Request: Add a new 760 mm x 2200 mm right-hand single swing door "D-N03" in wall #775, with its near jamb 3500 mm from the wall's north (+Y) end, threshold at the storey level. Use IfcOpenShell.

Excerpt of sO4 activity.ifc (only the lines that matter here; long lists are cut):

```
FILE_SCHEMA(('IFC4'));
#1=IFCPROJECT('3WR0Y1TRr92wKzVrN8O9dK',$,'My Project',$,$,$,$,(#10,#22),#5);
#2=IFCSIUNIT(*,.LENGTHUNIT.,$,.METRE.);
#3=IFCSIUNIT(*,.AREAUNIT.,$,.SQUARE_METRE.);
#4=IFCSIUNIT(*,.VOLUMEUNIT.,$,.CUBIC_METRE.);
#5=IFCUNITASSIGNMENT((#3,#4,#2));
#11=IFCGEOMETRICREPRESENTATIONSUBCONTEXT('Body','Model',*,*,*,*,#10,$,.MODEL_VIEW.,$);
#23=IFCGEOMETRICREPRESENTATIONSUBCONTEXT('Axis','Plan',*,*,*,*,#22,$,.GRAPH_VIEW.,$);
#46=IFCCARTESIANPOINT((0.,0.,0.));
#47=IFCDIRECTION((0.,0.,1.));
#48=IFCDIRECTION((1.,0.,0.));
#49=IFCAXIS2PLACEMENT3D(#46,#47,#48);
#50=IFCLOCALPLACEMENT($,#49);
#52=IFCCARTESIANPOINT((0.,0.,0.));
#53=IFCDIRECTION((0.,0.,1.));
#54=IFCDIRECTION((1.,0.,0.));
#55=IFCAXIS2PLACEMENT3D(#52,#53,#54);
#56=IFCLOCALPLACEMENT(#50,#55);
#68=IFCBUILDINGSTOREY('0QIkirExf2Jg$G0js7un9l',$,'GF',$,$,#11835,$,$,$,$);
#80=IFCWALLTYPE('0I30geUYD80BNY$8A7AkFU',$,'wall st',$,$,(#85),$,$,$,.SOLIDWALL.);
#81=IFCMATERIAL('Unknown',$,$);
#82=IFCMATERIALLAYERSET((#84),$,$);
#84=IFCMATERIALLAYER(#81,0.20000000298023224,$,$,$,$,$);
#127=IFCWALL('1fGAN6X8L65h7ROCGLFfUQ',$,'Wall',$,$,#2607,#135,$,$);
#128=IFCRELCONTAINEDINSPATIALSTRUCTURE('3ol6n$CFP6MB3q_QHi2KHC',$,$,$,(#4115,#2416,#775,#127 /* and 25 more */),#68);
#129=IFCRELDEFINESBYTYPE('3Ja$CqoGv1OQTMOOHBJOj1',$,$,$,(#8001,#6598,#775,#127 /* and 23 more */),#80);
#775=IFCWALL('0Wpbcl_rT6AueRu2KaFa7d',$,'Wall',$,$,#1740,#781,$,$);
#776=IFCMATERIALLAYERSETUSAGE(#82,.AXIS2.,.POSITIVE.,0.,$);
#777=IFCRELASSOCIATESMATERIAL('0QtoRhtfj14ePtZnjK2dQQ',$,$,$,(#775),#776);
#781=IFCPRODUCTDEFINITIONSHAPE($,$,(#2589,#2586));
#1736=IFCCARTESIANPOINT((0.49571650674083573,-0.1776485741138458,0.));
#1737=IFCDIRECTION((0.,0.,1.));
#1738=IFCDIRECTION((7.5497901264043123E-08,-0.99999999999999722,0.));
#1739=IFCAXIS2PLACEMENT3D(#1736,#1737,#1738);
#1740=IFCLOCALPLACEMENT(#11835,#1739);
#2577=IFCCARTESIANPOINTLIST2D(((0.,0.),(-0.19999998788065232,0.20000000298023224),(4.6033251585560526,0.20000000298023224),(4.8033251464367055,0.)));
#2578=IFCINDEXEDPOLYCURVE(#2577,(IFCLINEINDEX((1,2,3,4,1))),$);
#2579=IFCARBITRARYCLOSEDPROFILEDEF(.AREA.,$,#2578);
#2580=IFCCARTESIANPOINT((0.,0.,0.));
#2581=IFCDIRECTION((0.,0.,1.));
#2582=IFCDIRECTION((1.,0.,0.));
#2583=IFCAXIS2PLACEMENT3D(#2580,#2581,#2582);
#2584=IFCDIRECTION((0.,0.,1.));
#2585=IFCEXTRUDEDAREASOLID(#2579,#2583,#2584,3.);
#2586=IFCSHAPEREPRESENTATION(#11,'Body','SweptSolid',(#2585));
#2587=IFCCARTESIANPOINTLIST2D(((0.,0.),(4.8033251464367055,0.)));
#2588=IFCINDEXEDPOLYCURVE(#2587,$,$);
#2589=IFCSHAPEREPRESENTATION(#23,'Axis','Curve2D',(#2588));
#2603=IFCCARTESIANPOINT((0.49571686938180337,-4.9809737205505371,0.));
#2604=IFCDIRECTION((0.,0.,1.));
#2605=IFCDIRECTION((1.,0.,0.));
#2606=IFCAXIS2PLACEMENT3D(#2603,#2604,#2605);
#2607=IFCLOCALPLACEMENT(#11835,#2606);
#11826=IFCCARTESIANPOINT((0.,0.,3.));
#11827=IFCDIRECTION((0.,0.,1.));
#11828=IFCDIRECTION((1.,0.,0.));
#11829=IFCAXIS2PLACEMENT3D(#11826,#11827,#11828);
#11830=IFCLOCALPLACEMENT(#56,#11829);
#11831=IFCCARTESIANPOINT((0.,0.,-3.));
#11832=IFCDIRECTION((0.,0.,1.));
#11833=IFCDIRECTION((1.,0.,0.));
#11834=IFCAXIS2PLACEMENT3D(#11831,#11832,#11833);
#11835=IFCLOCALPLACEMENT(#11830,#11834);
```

```python
import numpy as np
import ifcopenshell
import ifcopenshell.api.feature
import ifcopenshell.api.geometry
import ifcopenshell.api.root
import ifcopenshell.api.spatial
import ifcopenshell.geom
import ifcopenshell.util.element
import ifcopenshell.util.placement
import ifcopenshell.util.representation
import ifcopenshell.util.shape
import ifcopenshell.util.unit

model = ifcopenshell.open("sO4 activity.ifc")
unit_scale = ifcopenshell.util.unit.calculate_unit_scale(model)
settings = ifcopenshell.geom.settings()


def volume(element):
    """Net volume in cubic metres, openings subtracted."""
    shape = ifcopenshell.geom.create_shape(settings, element)
    return ifcopenshell.util.shape.get_volume(shape.geometry)


wall = model.by_id(775)
storey = ifcopenshell.util.element.get_container(wall, ifc_class="IfcBuildingStorey")
context = ifcopenshell.util.representation.get_context(model, "Model", "Body", "MODEL_VIEW")
before = volume(wall)

width, height, from_end, sill = 0.76, 2.2, 3.5, 0.0  # metres

# The wall runs along its own X axis, and the end named is its -X end.
wall_shape = ifcopenshell.geom.create_shape(settings, wall)
x, y, z = ifcopenshell.util.shape.get_vertices(wall_shape.geometry).T
start = x.min() + from_end
face, thickness = float(y.min()), float(y.max() - y.min())
wall_matrix = ifcopenshell.util.placement.get_local_placement(wall.ObjectPlacement)
level = ifcopenshell.util.placement.get_local_placement(storey.ObjectPlacement)[2, 3]


def in_wall(x, y):
    """Placement at x, y metres in the wall's axes, at sill height."""
    matrix = wall_matrix.copy()
    matrix[:, 3] = wall_matrix @ np.array([x / unit_scale, y / unit_scale, 0.0, 1.0])
    matrix[2, 3] = level + sill / unit_scale
    return matrix


# Opening: a box that overshoots both wall faces by 50 mm.
opening = ifcopenshell.api.root.create_entity(model, ifc_class="IfcOpeningElement", predefined_type="OPENING")
box = ifcopenshell.api.geometry.add_wall_representation(
    model, context=context, length=width, height=height, thickness=thickness + 0.1
)
ifcopenshell.api.geometry.assign_representation(model, product=opening, representation=box)
ifcopenshell.api.geometry.edit_object_placement(model, product=opening, matrix=in_wall(start, face - 0.05), is_si=False)
ifcopenshell.api.feature.add_feature(model, feature=opening, element=wall)

door = ifcopenshell.api.root.create_entity(model, ifc_class="IfcDoor", name="D-N03", predefined_type="DOOR")
door.OverallWidth, door.OverallHeight = width / unit_scale, height / unit_scale
door.OperationType = "SINGLE_SWING_RIGHT"
body = ifcopenshell.api.geometry.add_door_representation(
    model,
    context=context,
    overall_width=door.OverallWidth,
    overall_height=door.OverallHeight,
    operation_type="SINGLE_SWING_RIGHT",
    lining_properties={"LiningDepth": thickness / unit_scale, "ThresholdDepth": thickness / unit_scale},
)
ifcopenshell.api.geometry.assign_representation(model, product=door, representation=body)
ifcopenshell.api.spatial.assign_container(model, products=[door], relating_structure=storey)
ifcopenshell.api.feature.add_filling(model, opening=opening, element=door)

# The lining spans the wall, so the door starts at the wall face.
ifcopenshell.api.geometry.edit_object_placement(model, product=door, matrix=in_wall(start, face), is_si=False)

after = volume(wall)

print(f"wall volume {before:.3f} -> {after:.3f} m3")

model.write("sO4 activity_edited.ifc")
```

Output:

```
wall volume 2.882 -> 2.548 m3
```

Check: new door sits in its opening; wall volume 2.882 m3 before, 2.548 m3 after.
